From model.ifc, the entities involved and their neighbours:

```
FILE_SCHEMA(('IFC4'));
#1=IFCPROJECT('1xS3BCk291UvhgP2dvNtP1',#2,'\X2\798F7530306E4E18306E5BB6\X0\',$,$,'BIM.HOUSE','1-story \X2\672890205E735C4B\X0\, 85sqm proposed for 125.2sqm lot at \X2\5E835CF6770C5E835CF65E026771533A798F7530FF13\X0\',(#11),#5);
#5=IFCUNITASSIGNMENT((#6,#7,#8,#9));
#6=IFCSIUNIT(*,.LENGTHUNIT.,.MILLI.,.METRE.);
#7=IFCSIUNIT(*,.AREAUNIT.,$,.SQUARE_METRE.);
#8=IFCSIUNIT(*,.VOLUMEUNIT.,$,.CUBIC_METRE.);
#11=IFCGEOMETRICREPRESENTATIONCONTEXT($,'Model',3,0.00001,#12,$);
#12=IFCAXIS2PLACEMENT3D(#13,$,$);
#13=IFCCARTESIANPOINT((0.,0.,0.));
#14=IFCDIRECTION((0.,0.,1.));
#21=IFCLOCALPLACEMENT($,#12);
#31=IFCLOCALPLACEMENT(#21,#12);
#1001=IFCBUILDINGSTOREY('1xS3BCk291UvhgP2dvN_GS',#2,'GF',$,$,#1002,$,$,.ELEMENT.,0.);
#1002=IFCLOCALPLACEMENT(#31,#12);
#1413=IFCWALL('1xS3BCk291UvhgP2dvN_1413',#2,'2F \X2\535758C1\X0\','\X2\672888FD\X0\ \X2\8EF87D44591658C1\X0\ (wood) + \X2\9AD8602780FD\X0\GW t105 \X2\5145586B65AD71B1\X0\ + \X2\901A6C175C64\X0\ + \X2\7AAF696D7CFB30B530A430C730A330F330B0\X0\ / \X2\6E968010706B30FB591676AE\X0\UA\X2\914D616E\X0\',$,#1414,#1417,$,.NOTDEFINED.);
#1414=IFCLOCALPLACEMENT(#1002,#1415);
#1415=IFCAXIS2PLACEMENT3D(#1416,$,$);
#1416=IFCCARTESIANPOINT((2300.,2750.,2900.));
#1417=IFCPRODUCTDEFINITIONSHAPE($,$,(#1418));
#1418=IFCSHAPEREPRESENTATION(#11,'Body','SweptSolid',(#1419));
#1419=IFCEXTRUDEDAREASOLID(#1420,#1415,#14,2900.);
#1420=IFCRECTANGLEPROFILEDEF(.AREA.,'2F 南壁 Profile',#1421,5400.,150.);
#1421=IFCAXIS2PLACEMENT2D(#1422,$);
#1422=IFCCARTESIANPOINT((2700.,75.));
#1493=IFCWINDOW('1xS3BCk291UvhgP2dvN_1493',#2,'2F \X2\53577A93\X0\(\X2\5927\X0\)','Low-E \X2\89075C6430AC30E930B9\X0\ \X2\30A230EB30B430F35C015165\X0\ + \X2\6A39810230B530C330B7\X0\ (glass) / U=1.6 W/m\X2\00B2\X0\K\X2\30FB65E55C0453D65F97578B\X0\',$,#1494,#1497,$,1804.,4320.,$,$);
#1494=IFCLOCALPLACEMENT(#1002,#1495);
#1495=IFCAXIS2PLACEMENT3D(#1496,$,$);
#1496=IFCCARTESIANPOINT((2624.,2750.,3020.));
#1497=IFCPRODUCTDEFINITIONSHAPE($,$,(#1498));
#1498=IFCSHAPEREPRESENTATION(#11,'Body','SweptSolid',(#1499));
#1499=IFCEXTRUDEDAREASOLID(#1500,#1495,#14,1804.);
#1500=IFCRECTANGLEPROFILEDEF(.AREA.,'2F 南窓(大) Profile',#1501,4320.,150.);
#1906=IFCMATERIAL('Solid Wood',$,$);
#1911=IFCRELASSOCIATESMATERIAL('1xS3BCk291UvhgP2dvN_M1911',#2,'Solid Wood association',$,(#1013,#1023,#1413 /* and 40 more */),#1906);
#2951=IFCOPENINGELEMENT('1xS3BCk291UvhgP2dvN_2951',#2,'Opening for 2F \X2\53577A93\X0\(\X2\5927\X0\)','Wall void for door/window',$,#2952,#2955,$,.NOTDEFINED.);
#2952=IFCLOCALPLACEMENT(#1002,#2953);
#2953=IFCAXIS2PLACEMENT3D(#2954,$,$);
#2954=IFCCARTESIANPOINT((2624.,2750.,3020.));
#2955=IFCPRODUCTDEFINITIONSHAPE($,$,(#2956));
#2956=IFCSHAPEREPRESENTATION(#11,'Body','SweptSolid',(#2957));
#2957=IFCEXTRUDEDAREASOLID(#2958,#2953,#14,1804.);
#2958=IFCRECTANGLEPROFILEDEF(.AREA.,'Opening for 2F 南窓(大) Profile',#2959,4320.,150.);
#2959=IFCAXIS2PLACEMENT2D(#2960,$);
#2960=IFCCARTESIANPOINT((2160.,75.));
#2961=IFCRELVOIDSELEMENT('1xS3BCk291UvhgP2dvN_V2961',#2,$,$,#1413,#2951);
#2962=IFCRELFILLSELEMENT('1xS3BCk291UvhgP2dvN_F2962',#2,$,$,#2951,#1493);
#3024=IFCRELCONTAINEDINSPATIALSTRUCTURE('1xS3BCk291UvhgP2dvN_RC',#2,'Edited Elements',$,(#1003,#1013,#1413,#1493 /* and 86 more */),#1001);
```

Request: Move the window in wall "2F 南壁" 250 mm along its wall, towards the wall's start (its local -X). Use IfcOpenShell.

```python
import ifcopenshell
import ifcopenshell.api.geometry
import ifcopenshell.util.placement
import ifcopenshell.util.unit

model = ifcopenshell.open("model.ifc")
unit_scale = ifcopenshell.util.unit.calculate_unit_scale(model)

window = model.by_id(1493)
opening = window.FillsVoids[0].RelatingOpeningElement
wall = opening.VoidsElements[0].RelatingBuildingElement

wall_matrix = ifcopenshell.util.placement.get_local_placement(wall.ObjectPlacement)
shift = wall_matrix[:3, 0] * -0.25 / unit_scale
before = ifcopenshell.util.placement.get_local_placement(window.ObjectPlacement)[:3, 3].copy()

# The window is not placed relative to its opening, so move both.
for product in (opening, window):
    matrix = ifcopenshell.util.placement.get_local_placement(product.ObjectPlacement)
    matrix[:3, 3] += shift
    ifcopenshell.api.geometry.edit_object_placement(model, product=product, matrix=matrix, is_si=False)

after = ifcopenshell.util.placement.get_local_placement(window.ObjectPlacement)[:3, 3]
print("window moved by", (after - before).round(3) + 0.0)

model.write("model_edited.ifc")
```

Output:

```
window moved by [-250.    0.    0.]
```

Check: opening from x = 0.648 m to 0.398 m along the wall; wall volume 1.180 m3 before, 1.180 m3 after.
